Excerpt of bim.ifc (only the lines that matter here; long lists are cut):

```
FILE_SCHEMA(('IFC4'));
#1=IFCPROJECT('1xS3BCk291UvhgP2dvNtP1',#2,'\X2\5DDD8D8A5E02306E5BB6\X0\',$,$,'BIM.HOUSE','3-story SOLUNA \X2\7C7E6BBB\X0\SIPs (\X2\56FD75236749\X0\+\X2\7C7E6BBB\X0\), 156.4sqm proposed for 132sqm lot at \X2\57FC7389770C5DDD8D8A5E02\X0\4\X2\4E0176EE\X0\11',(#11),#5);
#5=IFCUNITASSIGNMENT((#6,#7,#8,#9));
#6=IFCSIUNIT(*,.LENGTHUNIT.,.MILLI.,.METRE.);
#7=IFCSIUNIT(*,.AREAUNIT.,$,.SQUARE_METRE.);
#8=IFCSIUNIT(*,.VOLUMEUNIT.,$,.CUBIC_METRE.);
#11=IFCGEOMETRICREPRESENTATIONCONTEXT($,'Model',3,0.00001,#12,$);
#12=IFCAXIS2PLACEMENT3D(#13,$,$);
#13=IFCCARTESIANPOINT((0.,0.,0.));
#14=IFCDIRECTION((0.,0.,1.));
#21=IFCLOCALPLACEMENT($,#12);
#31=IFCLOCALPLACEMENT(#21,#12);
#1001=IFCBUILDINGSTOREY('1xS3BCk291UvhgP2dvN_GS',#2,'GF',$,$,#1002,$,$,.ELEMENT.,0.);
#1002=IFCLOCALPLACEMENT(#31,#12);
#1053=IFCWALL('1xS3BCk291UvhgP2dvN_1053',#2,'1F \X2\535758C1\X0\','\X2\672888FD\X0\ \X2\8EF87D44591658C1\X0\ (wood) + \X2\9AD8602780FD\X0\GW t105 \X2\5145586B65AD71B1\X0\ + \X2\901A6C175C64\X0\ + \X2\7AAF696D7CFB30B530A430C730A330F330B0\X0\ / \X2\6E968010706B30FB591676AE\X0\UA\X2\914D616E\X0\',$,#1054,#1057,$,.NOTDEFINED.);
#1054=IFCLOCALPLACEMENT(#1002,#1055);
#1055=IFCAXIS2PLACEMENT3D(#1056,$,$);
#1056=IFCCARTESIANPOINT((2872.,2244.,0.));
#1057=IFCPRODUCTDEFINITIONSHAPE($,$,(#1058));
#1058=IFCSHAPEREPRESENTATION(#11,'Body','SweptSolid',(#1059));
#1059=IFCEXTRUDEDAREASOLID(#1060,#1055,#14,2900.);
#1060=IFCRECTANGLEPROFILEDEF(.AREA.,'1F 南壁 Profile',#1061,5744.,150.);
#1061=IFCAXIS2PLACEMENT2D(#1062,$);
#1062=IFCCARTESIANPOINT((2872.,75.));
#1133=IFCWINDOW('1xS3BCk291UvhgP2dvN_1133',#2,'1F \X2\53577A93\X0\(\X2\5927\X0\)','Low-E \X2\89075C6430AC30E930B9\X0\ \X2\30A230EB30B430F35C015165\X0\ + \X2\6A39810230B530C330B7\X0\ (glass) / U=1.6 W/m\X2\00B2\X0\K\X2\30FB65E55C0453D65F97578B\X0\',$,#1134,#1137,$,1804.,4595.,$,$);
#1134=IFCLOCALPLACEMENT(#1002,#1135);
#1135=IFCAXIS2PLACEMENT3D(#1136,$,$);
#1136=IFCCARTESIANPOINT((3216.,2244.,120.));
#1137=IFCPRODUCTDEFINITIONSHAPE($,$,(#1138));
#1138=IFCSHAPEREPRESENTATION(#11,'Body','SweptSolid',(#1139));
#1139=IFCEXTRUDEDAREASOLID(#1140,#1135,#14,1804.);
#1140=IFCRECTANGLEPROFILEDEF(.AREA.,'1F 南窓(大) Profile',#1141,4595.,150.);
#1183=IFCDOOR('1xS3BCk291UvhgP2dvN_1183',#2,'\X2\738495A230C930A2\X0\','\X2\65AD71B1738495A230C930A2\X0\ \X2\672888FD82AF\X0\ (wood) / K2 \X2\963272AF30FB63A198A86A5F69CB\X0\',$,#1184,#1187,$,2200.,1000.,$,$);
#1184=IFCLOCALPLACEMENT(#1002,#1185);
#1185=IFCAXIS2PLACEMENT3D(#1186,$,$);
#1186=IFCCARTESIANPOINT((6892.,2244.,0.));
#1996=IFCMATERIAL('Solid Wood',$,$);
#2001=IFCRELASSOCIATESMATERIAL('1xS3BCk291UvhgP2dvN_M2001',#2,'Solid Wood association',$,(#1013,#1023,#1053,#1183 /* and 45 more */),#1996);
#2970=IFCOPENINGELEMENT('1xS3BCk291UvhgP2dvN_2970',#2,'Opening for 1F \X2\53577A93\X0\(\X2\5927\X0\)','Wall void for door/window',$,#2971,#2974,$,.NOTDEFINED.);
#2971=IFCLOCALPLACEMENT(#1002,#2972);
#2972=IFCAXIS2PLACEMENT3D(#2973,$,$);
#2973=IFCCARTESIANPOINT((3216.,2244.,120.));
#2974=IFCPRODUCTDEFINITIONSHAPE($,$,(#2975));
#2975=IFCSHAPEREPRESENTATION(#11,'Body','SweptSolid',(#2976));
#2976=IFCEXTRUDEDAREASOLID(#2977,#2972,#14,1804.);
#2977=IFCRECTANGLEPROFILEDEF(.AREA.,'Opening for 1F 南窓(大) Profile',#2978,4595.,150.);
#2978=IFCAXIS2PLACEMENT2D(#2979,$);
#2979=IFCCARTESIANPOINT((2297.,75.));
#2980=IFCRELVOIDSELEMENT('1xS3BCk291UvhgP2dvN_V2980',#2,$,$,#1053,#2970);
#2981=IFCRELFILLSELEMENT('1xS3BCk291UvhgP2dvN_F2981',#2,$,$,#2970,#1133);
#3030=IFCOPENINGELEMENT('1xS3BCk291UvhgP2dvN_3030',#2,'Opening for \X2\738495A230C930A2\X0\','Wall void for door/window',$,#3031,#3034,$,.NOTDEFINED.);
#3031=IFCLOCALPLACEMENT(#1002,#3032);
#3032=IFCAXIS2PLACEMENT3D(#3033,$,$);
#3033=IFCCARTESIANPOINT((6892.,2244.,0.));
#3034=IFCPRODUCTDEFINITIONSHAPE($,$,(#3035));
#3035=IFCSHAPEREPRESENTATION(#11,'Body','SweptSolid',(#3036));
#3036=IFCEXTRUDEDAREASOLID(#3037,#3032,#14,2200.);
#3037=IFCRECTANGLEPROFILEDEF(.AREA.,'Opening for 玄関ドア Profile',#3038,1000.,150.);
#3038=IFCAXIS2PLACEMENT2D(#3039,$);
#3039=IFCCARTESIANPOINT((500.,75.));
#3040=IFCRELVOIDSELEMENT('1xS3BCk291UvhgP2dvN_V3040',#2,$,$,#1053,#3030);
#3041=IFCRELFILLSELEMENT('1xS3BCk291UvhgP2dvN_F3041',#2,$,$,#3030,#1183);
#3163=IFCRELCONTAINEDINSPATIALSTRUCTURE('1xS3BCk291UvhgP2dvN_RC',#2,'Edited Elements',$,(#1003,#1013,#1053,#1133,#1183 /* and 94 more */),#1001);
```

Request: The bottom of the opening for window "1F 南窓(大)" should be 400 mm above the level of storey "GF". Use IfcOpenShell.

```python
import numpy as np
import ifcopenshell
import ifcopenshell.api.geometry
import ifcopenshell.geom
import ifcopenshell.util.element
import ifcopenshell.util.placement
import ifcopenshell.util.shape
import ifcopenshell.util.unit

model = ifcopenshell.open("bim.ifc")
unit_scale = ifcopenshell.util.unit.calculate_unit_scale(model)

window = model.by_guid("1xS3BCk291UvhgP2dvN_1133")
opening = window.FillsVoids[0].RelatingOpeningElement
storey = ifcopenshell.util.element.get_container(window, ifc_class="IfcBuildingStorey")
level = ifcopenshell.util.placement.get_local_placement(storey.ObjectPlacement)[2, 3]

# The opening's origin need not be at the sill, so measure its lowest point.
shape = ifcopenshell.geom.create_shape(ifcopenshell.geom.settings(), opening)
bottom = ifcopenshell.util.shape.get_shape_bottom_elevation(shape, shape.geometry) / unit_scale
dz = level + 0.4 / unit_scale - bottom

shift = np.array([0.0, 0.0, dz])
# The window is not placed relative to its opening, so move both.
for product in (opening, window):
    matrix = ifcopenshell.util.placement.get_local_placement(product.ObjectPlacement)
    matrix[:3, 3] += shift
    ifcopenshell.api.geometry.edit_object_placement(model, product=product, matrix=matrix, is_si=False)

print(f"moved by {dz * unit_scale:+.3f} m")

model.write("bim-out.ifc")
```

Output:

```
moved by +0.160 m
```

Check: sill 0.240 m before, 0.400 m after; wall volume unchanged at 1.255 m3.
